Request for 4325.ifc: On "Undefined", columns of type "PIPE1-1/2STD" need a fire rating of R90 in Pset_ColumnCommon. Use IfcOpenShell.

First a look at what the model holds.

```python
import ifcopenshell
import ifcopenshell.util.element

model = ifcopenshell.open("4325.ifc")
print(model.schema)
storey = next(s for s in model.by_type("IfcBuildingStorey") if s.Name == "Undefined")
columns = [e for e in ifcopenshell.util.element.get_decomposition(storey) if e.is_a("IfcColumn")]
seen = {}
for e in columns:
    element_type = ifcopenshell.util.element.get_type(e)
    key = (element_type.Name if element_type != e and element_type else None, ifcopenshell.util.element.get_pset(e, "Pset_ColumnCommon", "FireRating"))
    seen[key] = seen.get(key, 0) + 1
for (name, value), count in sorted(seen.items(), key=str):
    print(count, "x", name, "|", value)
```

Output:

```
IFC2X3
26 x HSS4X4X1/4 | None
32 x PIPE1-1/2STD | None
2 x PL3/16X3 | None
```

```python
import ifcopenshell
import ifcopenshell.api.pset
import ifcopenshell.util.element

model = ifcopenshell.open("4325.ifc")

storey = next(s for s in model.by_type("IfcBuildingStorey") if s.Name == "Undefined")
columns = [e for e in ifcopenshell.util.element.get_decomposition(storey) if e.is_a("IfcColumn")]

count = 0
for e in columns:
    element_type = ifcopenshell.util.element.get_type(e)
    if element_type in (None, e) or element_type.Name != "PIPE1-1/2STD":
        continue
    found = ifcopenshell.util.element.get_pset(e, "Pset_ColumnCommon", should_inherit=False)
    if found:
        pset = model.by_id(found["id"])
        if len(ifcopenshell.util.element.get_elements_by_pset(pset)) > 1:
            pset = ifcopenshell.api.pset.unshare_pset(model, products=[e], pset=pset)[0]
    else:
        pset = ifcopenshell.api.pset.add_pset(model, product=e, name="Pset_ColumnCommon")
    ifcopenshell.api.pset.edit_pset(model, pset=pset, properties={"FireRating": "R90"})
    count += 1

print(count, "columns updated")

model.write("4325_edited.ifc")
```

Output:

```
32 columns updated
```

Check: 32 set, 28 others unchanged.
